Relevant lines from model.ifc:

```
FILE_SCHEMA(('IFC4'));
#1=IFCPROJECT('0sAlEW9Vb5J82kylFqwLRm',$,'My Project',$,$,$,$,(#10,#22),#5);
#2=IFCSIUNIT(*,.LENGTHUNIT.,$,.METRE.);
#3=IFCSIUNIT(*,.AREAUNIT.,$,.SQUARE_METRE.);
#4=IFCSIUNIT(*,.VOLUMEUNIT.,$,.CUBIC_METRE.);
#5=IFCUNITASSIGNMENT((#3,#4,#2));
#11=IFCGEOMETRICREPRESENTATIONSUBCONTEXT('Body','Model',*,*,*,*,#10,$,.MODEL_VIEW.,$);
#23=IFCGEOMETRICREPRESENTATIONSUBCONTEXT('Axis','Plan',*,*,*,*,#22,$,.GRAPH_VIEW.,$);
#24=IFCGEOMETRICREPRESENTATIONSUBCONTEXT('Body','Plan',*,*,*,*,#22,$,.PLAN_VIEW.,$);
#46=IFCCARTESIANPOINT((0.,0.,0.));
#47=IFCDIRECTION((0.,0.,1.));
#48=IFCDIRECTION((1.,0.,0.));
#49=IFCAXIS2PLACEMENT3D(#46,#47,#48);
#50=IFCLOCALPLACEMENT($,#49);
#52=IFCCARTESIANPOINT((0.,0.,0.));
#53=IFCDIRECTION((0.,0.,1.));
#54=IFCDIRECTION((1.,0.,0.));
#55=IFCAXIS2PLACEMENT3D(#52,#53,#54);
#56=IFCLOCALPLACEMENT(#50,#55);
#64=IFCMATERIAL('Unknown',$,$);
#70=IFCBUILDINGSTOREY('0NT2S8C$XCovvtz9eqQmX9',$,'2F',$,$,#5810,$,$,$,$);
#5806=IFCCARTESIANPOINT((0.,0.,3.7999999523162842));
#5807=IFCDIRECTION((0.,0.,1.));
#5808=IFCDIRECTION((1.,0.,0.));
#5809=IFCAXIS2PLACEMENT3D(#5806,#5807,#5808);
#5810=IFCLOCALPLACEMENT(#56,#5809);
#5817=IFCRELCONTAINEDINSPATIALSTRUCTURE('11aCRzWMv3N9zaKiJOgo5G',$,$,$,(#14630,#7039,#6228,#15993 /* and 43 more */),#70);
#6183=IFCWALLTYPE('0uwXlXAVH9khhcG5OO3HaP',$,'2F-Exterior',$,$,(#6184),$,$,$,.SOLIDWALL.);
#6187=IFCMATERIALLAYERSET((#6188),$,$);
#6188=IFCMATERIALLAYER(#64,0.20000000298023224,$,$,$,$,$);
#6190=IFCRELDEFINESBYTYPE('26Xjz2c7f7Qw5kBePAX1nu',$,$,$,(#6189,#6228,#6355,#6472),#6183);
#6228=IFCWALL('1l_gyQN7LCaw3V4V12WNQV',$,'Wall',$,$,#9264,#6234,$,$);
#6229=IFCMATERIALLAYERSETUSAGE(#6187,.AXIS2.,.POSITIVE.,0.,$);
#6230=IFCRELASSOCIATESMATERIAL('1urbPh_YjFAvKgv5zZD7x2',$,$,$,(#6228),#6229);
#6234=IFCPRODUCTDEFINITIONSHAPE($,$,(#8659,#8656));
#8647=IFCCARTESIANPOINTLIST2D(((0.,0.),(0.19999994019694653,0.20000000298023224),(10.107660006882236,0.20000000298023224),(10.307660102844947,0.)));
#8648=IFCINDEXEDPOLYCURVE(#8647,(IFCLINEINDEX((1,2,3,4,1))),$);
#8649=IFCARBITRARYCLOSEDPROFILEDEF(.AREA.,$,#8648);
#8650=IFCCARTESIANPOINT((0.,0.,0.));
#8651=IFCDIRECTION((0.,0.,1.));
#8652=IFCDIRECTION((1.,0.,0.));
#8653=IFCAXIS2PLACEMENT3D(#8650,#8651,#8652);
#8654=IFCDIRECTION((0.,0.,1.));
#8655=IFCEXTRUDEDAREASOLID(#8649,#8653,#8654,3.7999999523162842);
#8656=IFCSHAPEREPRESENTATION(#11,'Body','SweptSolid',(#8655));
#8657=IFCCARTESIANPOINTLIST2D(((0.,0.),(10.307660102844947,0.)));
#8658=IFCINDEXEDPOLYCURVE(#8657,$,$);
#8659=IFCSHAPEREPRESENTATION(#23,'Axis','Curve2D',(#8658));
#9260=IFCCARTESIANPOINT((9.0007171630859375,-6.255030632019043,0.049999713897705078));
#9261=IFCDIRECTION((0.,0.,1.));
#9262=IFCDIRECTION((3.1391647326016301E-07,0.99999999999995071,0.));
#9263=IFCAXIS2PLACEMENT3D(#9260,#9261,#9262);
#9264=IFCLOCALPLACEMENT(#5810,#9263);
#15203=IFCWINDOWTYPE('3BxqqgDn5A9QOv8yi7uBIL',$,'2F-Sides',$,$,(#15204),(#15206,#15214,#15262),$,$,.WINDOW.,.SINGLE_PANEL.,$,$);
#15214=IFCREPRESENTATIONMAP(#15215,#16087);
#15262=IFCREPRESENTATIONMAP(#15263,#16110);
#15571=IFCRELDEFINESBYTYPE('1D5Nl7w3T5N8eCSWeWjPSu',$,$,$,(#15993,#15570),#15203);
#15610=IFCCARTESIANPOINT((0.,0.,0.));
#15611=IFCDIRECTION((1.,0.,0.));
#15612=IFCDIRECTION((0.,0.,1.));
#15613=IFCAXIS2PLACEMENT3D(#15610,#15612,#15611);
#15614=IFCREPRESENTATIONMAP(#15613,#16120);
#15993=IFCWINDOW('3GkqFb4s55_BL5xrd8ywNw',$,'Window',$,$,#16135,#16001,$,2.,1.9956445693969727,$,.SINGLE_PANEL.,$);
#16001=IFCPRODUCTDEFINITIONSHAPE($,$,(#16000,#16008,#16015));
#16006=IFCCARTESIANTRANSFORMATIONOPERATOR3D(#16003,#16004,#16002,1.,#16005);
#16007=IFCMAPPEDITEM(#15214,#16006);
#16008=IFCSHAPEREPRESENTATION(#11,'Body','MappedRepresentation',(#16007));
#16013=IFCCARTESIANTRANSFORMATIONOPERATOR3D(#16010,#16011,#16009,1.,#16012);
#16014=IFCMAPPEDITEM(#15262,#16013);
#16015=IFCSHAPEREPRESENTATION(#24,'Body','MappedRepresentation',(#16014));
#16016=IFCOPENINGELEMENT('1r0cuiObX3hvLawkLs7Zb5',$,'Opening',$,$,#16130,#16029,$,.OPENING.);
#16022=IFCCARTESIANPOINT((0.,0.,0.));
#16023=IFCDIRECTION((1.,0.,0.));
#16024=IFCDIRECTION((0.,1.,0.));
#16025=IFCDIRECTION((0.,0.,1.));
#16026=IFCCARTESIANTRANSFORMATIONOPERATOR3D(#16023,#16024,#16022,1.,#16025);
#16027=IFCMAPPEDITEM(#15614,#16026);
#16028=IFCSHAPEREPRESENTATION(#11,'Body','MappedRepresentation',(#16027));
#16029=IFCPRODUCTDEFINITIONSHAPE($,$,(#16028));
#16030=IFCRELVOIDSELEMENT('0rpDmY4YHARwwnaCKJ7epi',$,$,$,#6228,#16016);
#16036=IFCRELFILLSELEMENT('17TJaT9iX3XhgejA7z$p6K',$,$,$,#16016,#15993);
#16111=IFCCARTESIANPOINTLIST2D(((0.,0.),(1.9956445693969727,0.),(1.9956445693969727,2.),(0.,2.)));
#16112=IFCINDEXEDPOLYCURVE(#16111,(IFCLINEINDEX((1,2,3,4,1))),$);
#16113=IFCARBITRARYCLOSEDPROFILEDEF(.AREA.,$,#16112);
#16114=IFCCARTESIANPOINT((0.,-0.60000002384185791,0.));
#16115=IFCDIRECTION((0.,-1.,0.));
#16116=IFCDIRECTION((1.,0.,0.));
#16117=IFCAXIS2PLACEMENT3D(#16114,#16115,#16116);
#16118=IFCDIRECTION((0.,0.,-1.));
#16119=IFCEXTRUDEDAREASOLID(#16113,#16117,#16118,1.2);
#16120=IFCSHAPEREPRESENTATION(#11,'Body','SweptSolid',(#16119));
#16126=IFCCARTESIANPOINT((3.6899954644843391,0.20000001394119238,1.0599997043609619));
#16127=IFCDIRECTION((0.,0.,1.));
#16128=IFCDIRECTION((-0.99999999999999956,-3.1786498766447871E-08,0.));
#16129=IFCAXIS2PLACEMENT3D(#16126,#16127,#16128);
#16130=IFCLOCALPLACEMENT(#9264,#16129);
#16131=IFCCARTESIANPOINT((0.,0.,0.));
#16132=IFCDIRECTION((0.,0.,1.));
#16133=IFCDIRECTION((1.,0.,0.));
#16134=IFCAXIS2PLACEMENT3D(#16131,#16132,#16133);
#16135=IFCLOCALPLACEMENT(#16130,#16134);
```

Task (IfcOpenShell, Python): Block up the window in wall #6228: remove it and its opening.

```python
import ifcopenshell
import ifcopenshell.api.feature
import ifcopenshell.api.root
import ifcopenshell.geom
import ifcopenshell.util.shape

model = ifcopenshell.open("model.ifc")
settings = ifcopenshell.geom.settings()


def volume(element):
    """Net volume in cubic metres, openings subtracted."""
    shape = ifcopenshell.geom.create_shape(settings, element)
    return ifcopenshell.util.shape.get_volume(shape.geometry)


window = model.by_guid("3GkqFb4s55_BL5xrd8ywNw")
opening = window.FillsVoids[0].RelatingOpeningElement
wall = opening.VoidsElements[0].RelatingBuildingElement
before = volume(wall)

ifcopenshell.api.root.remove_product(model, product=window)
ifcopenshell.api.feature.remove_feature(model, feature=opening)

after = volume(wall)

print(f"wall volume {before:.3f} -> {after:.3f} m3")

model.write("model_updated.ifc")
```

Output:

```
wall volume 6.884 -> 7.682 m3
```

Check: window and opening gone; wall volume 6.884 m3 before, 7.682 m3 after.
